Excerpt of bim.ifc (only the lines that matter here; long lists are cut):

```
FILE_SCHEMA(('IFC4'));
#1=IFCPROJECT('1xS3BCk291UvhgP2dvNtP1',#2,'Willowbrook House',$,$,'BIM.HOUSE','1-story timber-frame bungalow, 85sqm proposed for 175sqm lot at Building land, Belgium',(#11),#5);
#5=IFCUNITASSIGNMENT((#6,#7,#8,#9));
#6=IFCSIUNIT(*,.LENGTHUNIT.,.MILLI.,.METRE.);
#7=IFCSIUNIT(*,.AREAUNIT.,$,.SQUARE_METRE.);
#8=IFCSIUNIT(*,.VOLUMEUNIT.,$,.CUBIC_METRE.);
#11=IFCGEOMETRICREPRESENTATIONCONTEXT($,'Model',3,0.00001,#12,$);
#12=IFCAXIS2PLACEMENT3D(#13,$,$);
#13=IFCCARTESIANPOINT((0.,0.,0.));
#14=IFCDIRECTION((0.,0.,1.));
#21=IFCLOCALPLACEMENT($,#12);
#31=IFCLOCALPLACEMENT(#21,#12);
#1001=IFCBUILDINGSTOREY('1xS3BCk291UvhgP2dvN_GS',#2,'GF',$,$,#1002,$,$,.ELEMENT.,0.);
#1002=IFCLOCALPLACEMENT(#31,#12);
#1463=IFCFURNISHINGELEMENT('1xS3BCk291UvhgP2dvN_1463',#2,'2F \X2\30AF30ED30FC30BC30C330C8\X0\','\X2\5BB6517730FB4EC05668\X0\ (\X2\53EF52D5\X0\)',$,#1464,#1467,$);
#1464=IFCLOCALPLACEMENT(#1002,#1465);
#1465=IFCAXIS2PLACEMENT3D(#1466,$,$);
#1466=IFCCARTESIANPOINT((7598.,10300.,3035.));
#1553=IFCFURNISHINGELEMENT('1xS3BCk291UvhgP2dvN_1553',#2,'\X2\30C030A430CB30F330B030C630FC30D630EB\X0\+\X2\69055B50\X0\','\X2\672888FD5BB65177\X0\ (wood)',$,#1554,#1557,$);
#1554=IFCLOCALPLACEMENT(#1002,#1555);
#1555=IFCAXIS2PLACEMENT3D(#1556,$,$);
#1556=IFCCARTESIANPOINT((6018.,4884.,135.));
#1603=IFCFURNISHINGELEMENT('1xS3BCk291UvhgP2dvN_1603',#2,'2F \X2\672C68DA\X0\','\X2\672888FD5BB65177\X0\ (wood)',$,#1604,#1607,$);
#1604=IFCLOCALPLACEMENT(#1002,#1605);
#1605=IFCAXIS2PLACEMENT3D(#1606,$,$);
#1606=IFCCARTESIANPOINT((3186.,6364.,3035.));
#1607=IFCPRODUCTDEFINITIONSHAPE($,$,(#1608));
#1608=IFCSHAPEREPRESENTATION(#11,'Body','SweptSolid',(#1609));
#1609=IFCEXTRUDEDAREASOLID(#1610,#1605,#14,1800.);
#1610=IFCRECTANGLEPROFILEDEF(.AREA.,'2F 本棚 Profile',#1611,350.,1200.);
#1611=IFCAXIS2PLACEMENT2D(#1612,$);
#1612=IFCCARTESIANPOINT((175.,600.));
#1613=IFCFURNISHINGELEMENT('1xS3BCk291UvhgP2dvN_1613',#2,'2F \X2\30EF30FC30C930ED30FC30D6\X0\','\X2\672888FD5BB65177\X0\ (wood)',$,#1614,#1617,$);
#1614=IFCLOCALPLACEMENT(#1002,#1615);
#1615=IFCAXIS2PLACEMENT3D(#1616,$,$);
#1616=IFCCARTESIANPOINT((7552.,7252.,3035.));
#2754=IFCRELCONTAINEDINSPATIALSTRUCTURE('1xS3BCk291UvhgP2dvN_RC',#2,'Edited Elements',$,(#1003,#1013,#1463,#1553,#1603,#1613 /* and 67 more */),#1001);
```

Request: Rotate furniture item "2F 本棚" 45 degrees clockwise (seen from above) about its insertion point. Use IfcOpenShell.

```python
import ifcopenshell
import ifcopenshell.api.geometry
import ifcopenshell.util.placement

model = ifcopenshell.open("bim.ifc")

item = model.by_guid("1xS3BCk291UvhgP2dvN_1603")
matrix = ifcopenshell.util.placement.get_local_placement(item.ObjectPlacement)
matrix = matrix @ ifcopenshell.util.placement.rotation(-45, "Z")
ifcopenshell.api.geometry.edit_object_placement(model, product=item, matrix=matrix, is_si=False)

print(ifcopenshell.util.placement.get_local_placement(item.ObjectPlacement).round(3) + 0.0)

model.write("bim_v2.ifc")
```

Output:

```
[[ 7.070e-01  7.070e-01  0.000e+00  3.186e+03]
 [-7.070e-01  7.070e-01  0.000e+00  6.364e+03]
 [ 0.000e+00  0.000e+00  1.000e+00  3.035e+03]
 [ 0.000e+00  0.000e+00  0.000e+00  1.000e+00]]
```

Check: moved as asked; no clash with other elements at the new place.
